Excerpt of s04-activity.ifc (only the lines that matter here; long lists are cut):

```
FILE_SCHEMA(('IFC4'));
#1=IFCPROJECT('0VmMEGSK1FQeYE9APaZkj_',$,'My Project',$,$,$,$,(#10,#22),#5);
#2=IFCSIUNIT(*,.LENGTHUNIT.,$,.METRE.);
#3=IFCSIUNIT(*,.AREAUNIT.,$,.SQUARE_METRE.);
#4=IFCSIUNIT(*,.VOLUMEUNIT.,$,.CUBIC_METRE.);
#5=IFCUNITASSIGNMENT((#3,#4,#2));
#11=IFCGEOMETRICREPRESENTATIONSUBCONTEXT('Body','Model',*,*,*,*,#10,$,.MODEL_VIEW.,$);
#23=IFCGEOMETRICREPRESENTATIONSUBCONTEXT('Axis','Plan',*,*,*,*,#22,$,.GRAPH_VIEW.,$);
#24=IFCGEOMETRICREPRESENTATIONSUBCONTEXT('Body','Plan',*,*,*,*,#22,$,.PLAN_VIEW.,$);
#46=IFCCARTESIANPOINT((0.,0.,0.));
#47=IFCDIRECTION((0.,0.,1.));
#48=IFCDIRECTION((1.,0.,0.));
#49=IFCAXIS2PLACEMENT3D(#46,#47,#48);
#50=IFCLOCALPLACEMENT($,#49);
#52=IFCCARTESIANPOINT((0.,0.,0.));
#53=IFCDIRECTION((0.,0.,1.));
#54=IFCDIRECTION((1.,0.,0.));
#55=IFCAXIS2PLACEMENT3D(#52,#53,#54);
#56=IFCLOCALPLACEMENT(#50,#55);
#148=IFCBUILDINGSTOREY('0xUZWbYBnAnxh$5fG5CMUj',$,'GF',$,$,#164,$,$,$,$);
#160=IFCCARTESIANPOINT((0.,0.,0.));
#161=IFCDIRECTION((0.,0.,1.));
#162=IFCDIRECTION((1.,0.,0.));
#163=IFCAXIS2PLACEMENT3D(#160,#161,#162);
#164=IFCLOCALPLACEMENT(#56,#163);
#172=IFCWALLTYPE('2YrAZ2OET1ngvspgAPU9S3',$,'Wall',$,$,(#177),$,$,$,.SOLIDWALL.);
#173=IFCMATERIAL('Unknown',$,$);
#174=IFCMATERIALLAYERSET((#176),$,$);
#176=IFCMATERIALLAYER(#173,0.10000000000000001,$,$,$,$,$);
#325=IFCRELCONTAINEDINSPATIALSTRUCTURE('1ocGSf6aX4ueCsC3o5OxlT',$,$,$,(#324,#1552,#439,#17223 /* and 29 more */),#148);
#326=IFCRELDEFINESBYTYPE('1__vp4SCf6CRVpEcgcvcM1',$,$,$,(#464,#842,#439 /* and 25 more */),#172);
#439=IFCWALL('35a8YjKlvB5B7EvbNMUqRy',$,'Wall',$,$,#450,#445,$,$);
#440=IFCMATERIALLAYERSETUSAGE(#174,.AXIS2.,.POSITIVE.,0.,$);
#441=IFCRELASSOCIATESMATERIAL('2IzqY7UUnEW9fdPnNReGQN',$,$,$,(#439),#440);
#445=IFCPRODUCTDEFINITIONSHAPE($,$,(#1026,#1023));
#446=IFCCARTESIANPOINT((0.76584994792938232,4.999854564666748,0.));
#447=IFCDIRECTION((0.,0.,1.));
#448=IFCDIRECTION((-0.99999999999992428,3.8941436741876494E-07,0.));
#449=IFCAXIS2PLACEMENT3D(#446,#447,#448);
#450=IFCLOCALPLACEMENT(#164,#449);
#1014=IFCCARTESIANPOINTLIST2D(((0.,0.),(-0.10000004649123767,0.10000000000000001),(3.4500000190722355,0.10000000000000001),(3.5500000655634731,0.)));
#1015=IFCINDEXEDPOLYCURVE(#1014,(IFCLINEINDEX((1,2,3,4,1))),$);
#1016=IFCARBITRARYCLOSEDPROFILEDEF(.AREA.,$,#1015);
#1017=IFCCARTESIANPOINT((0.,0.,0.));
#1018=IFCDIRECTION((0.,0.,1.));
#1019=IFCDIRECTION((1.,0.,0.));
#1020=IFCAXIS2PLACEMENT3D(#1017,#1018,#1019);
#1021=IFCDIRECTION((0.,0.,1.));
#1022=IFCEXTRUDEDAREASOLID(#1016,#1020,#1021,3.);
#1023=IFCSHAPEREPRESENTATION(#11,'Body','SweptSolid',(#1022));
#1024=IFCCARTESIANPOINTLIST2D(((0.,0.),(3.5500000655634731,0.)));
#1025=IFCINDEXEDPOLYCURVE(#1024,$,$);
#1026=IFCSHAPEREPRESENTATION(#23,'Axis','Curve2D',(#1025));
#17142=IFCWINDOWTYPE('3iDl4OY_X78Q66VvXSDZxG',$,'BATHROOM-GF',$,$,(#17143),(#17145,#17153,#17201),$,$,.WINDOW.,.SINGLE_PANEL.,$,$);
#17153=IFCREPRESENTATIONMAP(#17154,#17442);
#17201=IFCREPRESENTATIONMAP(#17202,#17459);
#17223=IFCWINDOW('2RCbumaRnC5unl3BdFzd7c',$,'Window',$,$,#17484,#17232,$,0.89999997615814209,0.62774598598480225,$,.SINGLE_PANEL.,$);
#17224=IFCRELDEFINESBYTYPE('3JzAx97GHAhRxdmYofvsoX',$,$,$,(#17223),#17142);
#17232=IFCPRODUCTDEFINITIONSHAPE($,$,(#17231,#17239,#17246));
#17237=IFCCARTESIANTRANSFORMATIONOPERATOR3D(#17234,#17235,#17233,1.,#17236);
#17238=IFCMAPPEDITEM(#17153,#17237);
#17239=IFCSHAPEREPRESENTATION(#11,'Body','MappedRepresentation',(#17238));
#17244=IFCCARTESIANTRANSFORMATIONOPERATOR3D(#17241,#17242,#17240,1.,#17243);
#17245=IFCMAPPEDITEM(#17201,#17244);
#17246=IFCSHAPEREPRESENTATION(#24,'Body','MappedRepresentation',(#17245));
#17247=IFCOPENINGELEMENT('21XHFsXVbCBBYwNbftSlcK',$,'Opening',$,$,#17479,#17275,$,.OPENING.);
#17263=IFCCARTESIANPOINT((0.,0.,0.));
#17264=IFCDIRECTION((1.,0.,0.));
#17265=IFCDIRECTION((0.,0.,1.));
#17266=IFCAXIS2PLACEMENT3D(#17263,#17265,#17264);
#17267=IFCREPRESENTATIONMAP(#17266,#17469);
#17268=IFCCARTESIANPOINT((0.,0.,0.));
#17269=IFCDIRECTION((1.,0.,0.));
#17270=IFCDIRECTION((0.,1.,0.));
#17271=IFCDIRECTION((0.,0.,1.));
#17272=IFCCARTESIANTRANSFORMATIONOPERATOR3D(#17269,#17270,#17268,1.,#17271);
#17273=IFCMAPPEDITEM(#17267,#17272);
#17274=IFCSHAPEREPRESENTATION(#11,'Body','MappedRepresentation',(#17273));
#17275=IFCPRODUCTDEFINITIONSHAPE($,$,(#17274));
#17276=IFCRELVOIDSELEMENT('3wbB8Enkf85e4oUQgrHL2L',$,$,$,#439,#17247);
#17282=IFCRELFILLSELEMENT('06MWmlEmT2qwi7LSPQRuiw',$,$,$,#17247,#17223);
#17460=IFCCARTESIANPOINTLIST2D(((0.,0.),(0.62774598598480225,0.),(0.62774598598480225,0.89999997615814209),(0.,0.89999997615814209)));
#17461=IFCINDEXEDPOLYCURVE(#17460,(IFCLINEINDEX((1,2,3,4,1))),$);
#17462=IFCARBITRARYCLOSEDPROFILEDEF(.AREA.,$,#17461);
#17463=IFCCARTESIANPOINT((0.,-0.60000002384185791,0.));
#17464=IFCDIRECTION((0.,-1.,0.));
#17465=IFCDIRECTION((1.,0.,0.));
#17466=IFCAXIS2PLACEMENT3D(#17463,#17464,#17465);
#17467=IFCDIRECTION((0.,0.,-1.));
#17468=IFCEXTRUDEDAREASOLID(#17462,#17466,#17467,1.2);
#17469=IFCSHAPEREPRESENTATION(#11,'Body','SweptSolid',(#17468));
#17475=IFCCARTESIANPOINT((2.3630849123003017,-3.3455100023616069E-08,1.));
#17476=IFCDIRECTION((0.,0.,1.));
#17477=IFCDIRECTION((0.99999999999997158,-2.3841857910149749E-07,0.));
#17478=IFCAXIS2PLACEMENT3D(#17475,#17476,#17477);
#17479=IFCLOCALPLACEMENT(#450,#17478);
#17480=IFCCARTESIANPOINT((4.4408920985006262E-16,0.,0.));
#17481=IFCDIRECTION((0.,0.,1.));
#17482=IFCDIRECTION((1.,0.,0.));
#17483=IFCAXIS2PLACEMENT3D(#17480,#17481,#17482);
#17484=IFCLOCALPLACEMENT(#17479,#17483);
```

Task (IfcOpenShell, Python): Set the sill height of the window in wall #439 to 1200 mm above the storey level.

```python
import numpy as np
import ifcopenshell
import ifcopenshell.api.geometry
import ifcopenshell.geom
import ifcopenshell.util.element
import ifcopenshell.util.placement
import ifcopenshell.util.shape
import ifcopenshell.util.unit

model = ifcopenshell.open("s04-activity.ifc")
unit_scale = ifcopenshell.util.unit.calculate_unit_scale(model)

window = model.by_guid("2RCbumaRnC5unl3BdFzd7c")
opening = window.FillsVoids[0].RelatingOpeningElement
storey = ifcopenshell.util.element.get_container(window, ifc_class="IfcBuildingStorey")
level = ifcopenshell.util.placement.get_local_placement(storey.ObjectPlacement)[2, 3]

# The opening's origin need not be at the sill, so measure its lowest point.
shape = ifcopenshell.geom.create_shape(ifcopenshell.geom.settings(), opening)
bottom = ifcopenshell.util.shape.get_shape_bottom_elevation(shape, shape.geometry) / unit_scale
dz = level + 1.2 / unit_scale - bottom

shift = np.array([0.0, 0.0, dz])
# The window is placed relative to its opening, so it follows when the opening moves.
matrix = ifcopenshell.util.placement.get_local_placement(opening.ObjectPlacement)
matrix[:3, 3] += shift
ifcopenshell.api.geometry.edit_object_placement(
    model, product=opening, matrix=matrix, is_si=False, should_transform_children=True
)

print(f"moved by {dz * unit_scale:+.3f} m")

model.write("s04-activity_updated.ifc")
```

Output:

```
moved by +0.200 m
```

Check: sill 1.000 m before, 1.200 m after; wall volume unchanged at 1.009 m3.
